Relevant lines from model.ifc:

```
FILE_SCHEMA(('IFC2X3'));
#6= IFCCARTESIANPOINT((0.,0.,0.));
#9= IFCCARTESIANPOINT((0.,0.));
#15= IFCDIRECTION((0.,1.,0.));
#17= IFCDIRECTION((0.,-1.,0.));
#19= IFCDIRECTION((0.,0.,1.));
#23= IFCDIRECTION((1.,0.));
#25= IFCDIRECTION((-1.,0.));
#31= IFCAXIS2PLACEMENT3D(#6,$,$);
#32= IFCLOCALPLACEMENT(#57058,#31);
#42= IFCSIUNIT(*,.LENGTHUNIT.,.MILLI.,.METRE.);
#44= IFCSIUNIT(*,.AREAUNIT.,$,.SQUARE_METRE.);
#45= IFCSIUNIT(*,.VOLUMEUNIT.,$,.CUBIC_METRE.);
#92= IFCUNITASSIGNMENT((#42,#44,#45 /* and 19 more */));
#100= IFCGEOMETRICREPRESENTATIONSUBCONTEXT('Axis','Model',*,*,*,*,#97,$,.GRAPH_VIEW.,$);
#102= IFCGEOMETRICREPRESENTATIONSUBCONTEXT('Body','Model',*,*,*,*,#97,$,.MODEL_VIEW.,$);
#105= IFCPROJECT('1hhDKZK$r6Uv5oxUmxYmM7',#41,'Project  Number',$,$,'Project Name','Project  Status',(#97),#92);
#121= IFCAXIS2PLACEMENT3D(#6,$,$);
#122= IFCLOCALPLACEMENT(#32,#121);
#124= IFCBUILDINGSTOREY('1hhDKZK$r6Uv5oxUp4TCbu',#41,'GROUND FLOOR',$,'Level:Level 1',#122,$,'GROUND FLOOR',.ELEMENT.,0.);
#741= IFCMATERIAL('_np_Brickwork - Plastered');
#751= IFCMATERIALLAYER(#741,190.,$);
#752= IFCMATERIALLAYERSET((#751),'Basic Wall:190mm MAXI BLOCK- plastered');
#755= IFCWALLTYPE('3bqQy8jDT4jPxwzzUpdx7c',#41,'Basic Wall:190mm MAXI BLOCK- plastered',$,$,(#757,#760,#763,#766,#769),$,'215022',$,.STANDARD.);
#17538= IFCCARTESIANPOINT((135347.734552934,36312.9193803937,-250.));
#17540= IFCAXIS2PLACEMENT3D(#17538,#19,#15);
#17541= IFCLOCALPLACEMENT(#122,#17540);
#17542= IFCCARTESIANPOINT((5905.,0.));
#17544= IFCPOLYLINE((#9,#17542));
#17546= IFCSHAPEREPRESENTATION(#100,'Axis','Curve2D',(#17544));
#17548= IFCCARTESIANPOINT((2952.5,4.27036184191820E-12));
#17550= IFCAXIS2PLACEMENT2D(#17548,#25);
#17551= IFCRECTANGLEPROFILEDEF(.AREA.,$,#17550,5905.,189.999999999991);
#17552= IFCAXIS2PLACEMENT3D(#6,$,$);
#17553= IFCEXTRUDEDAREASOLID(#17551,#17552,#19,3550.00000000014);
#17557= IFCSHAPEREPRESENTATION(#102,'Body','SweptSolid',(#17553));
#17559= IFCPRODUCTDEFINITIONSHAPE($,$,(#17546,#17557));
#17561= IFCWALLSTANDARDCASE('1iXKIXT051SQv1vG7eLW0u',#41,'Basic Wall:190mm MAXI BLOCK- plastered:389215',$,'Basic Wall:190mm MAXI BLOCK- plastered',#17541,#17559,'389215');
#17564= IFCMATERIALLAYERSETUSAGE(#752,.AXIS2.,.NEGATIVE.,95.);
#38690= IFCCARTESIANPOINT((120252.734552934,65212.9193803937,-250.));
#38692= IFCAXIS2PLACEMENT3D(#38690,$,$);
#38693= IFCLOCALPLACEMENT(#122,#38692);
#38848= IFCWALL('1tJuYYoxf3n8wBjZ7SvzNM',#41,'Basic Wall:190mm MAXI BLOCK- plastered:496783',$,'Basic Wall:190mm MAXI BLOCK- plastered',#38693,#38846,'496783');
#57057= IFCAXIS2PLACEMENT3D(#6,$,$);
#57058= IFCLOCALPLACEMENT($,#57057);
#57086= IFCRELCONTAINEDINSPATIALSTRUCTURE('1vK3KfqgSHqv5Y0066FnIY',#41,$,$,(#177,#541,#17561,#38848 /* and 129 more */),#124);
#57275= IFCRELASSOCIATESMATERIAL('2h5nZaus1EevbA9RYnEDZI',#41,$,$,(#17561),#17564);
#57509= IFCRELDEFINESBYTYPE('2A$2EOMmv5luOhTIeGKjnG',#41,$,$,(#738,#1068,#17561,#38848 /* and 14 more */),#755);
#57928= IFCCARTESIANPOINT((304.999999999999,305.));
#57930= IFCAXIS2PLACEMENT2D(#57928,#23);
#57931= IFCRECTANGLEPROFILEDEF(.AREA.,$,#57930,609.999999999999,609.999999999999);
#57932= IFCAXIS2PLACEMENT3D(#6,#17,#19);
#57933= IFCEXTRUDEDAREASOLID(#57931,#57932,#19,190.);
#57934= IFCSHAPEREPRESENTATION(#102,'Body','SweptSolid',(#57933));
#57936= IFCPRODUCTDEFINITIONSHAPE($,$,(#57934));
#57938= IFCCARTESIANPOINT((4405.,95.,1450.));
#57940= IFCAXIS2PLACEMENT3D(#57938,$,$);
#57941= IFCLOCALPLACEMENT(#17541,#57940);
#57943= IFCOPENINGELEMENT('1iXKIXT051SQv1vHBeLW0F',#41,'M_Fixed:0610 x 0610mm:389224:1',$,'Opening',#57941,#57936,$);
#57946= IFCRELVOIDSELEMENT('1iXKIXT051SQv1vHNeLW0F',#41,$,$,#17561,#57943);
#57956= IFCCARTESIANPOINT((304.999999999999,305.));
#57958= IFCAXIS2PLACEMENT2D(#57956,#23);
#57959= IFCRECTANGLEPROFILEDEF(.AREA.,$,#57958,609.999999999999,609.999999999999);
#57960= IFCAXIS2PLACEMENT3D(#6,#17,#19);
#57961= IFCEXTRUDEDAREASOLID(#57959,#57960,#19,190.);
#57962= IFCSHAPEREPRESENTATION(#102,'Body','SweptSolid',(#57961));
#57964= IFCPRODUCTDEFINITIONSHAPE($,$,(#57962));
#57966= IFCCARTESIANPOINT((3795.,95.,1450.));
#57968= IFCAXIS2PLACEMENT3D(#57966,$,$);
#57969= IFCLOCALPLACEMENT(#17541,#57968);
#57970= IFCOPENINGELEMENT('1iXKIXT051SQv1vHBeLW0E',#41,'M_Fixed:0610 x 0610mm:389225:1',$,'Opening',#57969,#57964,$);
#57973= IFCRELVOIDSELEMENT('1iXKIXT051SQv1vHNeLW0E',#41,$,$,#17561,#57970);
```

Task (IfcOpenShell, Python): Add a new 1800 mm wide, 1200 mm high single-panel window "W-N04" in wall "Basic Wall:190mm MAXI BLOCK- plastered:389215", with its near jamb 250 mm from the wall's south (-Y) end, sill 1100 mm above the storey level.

```python
import numpy as np
import ifcopenshell
import ifcopenshell.api.feature
import ifcopenshell.api.geometry
import ifcopenshell.api.root
import ifcopenshell.api.spatial
import ifcopenshell.api.type
import ifcopenshell.geom
import ifcopenshell.util.element
import ifcopenshell.util.placement
import ifcopenshell.util.representation
import ifcopenshell.util.shape
import ifcopenshell.util.unit

model = ifcopenshell.open("model.ifc")
unit_scale = ifcopenshell.util.unit.calculate_unit_scale(model)
settings = ifcopenshell.geom.settings()


def volume(element):
    """Net volume in cubic metres, openings subtracted."""
    shape = ifcopenshell.geom.create_shape(settings, element)
    return ifcopenshell.util.shape.get_volume(shape.geometry)


wall = model.by_guid("1iXKIXT051SQv1vG7eLW0u")
storey = ifcopenshell.util.element.get_container(wall, ifc_class="IfcBuildingStorey")
context = ifcopenshell.util.representation.get_context(model, "Model", "Body", "MODEL_VIEW")
before = volume(wall)

width, height, from_end, sill = 1.8, 1.2, 0.25, 1.1  # metres

# The wall runs along its own X axis, and the end named is its -X end.
wall_shape = ifcopenshell.geom.create_shape(settings, wall)
x, y, z = ifcopenshell.util.shape.get_vertices(wall_shape.geometry).T
start = x.min() + from_end
face, thickness = float(y.min()), float(y.max() - y.min())
wall_matrix = ifcopenshell.util.placement.get_local_placement(wall.ObjectPlacement)
level = ifcopenshell.util.placement.get_local_placement(storey.ObjectPlacement)[2, 3]


def in_wall(x, y):
    """Placement at x, y metres in the wall's axes, at sill height."""
    matrix = wall_matrix.copy()
    matrix[:, 3] = wall_matrix @ np.array([x / unit_scale, y / unit_scale, 0.0, 1.0])
    matrix[2, 3] = level + sill / unit_scale
    return matrix


# Opening: a box that overshoots both wall faces by 50 mm.
opening = ifcopenshell.api.root.create_entity(model, ifc_class="IfcOpeningElement")
box = ifcopenshell.api.geometry.add_wall_representation(
    model, context=context, length=width, height=height, thickness=thickness + 0.1
)
ifcopenshell.api.geometry.assign_representation(model, product=opening, representation=box)
ifcopenshell.api.geometry.edit_object_placement(model, product=opening, matrix=in_wall(start, face - 0.05), is_si=False)
ifcopenshell.api.feature.add_feature(model, feature=opening, element=wall)

window = ifcopenshell.api.root.create_entity(model, ifc_class="IfcWindow", name="W-N04")
window.OverallWidth, window.OverallHeight = width / unit_scale, height / unit_scale
body = ifcopenshell.api.geometry.add_window_representation(
    model,
    context=context,
    overall_width=window.OverallWidth,
    overall_height=window.OverallHeight,
    partition_type="SINGLE_PANEL",
)
ifcopenshell.api.geometry.assign_representation(model, product=window, representation=body)
ifcopenshell.api.spatial.assign_container(model, products=[window], relating_structure=storey)
fills = ifcopenshell.api.feature.add_filling(model, opening=opening, element=window)
fills.OwnerHistory = window.OwnerHistory  # required in IFC2X3

# IFC2X3 keeps the operation on the window style.
style = ifcopenshell.api.root.create_entity(model, ifc_class="IfcWindowStyle", name="W-N04")
style.OperationType, style.ConstructionType = "SINGLE_PANEL", "NOTDEFINED"
style.ParameterTakesPrecedence = style.Sizeable = False
ifcopenshell.api.type.assign_type(model, related_objects=[window], relating_type=style)

# Centre the window in the wall's thickness.
ifcopenshell.api.geometry.edit_object_placement(model, product=window, matrix=in_wall(start, face), is_si=False)
window_shape = ifcopenshell.geom.create_shape(settings, window)
depth = ifcopenshell.util.shape.get_vertices(window_shape.geometry)[:, 1]
offset = face + thickness / 2 - (depth.min() + depth.max()) / 2
ifcopenshell.api.geometry.edit_object_placement(model, product=window, matrix=in_wall(start, offset), is_si=False)

after = volume(wall)

print(f"wall volume {before:.3f} -> {after:.3f} m3")

model.write("model_updated.ifc")
```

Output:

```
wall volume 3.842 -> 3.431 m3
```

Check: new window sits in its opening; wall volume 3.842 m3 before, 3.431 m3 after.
